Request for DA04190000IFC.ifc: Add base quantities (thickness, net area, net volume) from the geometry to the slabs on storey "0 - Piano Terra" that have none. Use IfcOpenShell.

First a look at what the model holds.

```python
import ifcopenshell
import ifcopenshell.util.element
import ifcopenshell.util.unit

model = ifcopenshell.open("DA04190000IFC.ifc")
print(model.schema)
for unit_type in ("LENGTHUNIT", "AREAUNIT", "VOLUMEUNIT"):
    print(unit_type, ifcopenshell.util.unit.calculate_unit_scale(model, unit_type))
storey = next(s for s in model.by_type("IfcBuildingStorey") if s.Name == "0 - Piano Terra")
slabs = [e for e in ifcopenshell.util.element.get_decomposition(storey) if e.is_a("IfcSlab")]
for e in sorted(slabs, key=lambda e: e.id()):
    print(e.id(), e.is_a(), e.Name, list(ifcopenshell.util.element.get_psets(e, qtos_only=True)), sep=" | ")
```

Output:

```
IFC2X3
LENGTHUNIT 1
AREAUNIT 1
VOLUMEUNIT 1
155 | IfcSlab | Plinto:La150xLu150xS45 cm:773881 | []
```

```python
import ifcopenshell
import ifcopenshell.api.pset
import ifcopenshell.geom
import ifcopenshell.util.element
import ifcopenshell.util.shape
import ifcopenshell.util.unit

model = ifcopenshell.open("DA04190000IFC.ifc")
unit_scale = ifcopenshell.util.unit.calculate_unit_scale(model)
area_scale = ifcopenshell.util.unit.calculate_unit_scale(model, "AREAUNIT")
volume_scale = ifcopenshell.util.unit.calculate_unit_scale(model, "VOLUMEUNIT")
settings = ifcopenshell.geom.settings()

storey = next(s for s in model.by_type("IfcBuildingStorey") if s.Name == "0 - Piano Terra")
slabs = [e for e in ifcopenshell.util.element.get_decomposition(storey) if e.is_a("IfcSlab")]

for e in sorted(slabs, key=lambda e: e.id()):
    if ifcopenshell.util.element.get_psets(e, qtos_only=True, should_inherit=False):
        continue
    # Geometry comes back in metres, in the element's own axes.
    shape = ifcopenshell.geom.create_shape(settings, e)
    values = {
        "Width": ifcopenshell.util.shape.get_z(shape.geometry) / unit_scale,
        "NetArea": ifcopenshell.util.shape.get_footprint_area(shape.geometry) / area_scale,
        "NetVolume": ifcopenshell.util.shape.get_volume(shape.geometry) / volume_scale,
    }
    qto = ifcopenshell.api.pset.add_qto(model, product=e, name="BaseQuantities")
    ifcopenshell.api.pset.edit_qto(model, qto=qto, properties=values)
    print(e.id(), {k: round(v, 3) for k, v in values.items()})

model.write("DA04190000IFC-out.ifc")
```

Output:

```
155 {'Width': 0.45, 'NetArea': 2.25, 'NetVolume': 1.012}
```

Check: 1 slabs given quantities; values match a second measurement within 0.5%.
